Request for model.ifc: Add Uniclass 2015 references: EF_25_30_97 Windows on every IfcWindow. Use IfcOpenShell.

First a look at what the model holds.

```python
import ifcopenshell

model = ifcopenshell.open("model.ifc")
print(model.schema)
print("classifications:", [c.Name for c in model.by_type("IfcClassification")])
for ifc_class in ("IfcDoor", "IfcRoof", "IfcStair", "IfcWall", "IfcWindow"):
    print(ifc_class, len(model.by_type(ifc_class)))
```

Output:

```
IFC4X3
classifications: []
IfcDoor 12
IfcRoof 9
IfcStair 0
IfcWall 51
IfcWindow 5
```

```python
import ifcopenshell
import ifcopenshell.api.classification

model = ifcopenshell.open("model.ifc")

system = ifcopenshell.api.classification.add_classification(model, classification="Uniclass 2015")

codes = {
    "IfcWindow": ("EF_25_30_97", "Windows"),
}
for ifc_class, (code, name) in codes.items():
    products = model.by_type(ifc_class)
    ifcopenshell.api.classification.add_reference(
        model, products=products, classification=system, identification=code, name=name
    )
    print(code, len(products))

model.write("model_edited.ifc")
```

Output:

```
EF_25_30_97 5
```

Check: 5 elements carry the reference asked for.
